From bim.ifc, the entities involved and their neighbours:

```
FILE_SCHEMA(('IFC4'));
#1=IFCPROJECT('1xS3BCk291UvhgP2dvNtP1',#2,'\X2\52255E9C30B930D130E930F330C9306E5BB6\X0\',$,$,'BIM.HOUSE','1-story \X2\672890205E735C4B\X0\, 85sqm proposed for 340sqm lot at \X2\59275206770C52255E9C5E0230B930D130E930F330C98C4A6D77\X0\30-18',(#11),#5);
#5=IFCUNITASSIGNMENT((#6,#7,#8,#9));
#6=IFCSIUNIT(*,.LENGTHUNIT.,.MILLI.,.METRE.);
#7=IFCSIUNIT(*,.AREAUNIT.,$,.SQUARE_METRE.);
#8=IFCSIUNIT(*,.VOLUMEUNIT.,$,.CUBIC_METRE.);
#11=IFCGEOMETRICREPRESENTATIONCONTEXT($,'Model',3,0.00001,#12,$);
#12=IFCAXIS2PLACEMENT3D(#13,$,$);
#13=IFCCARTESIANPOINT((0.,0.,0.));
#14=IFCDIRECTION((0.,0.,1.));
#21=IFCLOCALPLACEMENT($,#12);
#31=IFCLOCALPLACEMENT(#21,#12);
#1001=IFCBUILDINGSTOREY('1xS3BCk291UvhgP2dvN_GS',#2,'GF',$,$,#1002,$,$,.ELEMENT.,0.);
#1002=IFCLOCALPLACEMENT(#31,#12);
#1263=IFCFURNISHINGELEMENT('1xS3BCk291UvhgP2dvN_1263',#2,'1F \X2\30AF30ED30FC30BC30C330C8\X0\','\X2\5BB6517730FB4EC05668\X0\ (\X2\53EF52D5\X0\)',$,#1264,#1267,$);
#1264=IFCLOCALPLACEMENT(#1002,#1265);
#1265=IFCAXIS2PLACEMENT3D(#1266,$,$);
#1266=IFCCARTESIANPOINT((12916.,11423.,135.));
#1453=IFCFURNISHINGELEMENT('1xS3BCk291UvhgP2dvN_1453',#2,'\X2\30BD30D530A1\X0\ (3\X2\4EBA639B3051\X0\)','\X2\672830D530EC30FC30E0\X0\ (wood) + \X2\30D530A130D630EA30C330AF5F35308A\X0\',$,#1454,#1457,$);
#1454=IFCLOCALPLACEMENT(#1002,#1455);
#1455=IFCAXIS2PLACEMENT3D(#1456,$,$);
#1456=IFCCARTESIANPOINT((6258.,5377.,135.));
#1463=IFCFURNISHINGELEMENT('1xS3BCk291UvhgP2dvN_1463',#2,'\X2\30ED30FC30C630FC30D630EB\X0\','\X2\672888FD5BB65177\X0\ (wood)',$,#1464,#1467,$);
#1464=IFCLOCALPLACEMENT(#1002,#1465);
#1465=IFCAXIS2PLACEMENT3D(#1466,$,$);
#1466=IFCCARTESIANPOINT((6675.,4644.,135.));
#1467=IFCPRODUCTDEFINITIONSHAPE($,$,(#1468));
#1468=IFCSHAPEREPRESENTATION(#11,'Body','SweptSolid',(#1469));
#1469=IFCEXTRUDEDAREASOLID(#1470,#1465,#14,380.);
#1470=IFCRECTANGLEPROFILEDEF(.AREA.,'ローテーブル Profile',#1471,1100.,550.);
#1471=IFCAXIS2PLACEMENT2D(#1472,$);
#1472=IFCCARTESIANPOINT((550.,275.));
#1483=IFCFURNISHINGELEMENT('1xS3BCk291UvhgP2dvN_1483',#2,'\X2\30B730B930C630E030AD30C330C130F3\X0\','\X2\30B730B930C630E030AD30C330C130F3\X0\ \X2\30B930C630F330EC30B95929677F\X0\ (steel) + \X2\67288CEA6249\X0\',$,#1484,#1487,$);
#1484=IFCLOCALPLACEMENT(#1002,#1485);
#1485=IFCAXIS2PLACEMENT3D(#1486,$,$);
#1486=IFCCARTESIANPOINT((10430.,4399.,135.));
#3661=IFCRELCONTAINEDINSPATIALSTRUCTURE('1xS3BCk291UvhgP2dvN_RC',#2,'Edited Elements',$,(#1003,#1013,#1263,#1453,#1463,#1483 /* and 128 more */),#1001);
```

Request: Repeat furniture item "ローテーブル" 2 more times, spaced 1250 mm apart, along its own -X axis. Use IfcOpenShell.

```python
import ifcopenshell
import ifcopenshell.api.geometry
import ifcopenshell.api.root
import ifcopenshell.util.element
import ifcopenshell.util.placement

model = ifcopenshell.open("bim.ifc")


def reuse_history(source, copy):
    """copy_class also copies each property set's owner history, people and application; keep the originals."""
    for rel in copy.IsDefinedBy:
        if rel.is_a("IfcRelDefinesByProperties") and (history := rel.RelatingPropertyDefinition.OwnerHistory):
            rel.RelatingPropertyDefinition.OwnerHistory = source.OwnerHistory
            ifcopenshell.util.element.remove_deep2(model, history)


source = model.by_id(1463)
base = ifcopenshell.util.placement.get_local_placement(source.ObjectPlacement)
step = -base[:3, 0] * 1250.0

for i in range(1, 3):
    copy = ifcopenshell.api.root.copy_class(model, product=source)
    copy.Representation = ifcopenshell.util.element.copy_deep(
        model, source.Representation, exclude=["IfcGeometricRepresentationContext", "IfcRepresentationMap"]
    )
    reuse_history(source, copy)
    matrix = base.copy()
    matrix[:3, 3] += i * step
    print("added at", matrix[:3, 3].round(3) + 0.0)
    ifcopenshell.api.geometry.edit_object_placement(model, product=copy, matrix=matrix, is_si=False)

model.write("bim_v2.ifc")
```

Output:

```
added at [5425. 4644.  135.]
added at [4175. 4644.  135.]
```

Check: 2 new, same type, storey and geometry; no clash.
